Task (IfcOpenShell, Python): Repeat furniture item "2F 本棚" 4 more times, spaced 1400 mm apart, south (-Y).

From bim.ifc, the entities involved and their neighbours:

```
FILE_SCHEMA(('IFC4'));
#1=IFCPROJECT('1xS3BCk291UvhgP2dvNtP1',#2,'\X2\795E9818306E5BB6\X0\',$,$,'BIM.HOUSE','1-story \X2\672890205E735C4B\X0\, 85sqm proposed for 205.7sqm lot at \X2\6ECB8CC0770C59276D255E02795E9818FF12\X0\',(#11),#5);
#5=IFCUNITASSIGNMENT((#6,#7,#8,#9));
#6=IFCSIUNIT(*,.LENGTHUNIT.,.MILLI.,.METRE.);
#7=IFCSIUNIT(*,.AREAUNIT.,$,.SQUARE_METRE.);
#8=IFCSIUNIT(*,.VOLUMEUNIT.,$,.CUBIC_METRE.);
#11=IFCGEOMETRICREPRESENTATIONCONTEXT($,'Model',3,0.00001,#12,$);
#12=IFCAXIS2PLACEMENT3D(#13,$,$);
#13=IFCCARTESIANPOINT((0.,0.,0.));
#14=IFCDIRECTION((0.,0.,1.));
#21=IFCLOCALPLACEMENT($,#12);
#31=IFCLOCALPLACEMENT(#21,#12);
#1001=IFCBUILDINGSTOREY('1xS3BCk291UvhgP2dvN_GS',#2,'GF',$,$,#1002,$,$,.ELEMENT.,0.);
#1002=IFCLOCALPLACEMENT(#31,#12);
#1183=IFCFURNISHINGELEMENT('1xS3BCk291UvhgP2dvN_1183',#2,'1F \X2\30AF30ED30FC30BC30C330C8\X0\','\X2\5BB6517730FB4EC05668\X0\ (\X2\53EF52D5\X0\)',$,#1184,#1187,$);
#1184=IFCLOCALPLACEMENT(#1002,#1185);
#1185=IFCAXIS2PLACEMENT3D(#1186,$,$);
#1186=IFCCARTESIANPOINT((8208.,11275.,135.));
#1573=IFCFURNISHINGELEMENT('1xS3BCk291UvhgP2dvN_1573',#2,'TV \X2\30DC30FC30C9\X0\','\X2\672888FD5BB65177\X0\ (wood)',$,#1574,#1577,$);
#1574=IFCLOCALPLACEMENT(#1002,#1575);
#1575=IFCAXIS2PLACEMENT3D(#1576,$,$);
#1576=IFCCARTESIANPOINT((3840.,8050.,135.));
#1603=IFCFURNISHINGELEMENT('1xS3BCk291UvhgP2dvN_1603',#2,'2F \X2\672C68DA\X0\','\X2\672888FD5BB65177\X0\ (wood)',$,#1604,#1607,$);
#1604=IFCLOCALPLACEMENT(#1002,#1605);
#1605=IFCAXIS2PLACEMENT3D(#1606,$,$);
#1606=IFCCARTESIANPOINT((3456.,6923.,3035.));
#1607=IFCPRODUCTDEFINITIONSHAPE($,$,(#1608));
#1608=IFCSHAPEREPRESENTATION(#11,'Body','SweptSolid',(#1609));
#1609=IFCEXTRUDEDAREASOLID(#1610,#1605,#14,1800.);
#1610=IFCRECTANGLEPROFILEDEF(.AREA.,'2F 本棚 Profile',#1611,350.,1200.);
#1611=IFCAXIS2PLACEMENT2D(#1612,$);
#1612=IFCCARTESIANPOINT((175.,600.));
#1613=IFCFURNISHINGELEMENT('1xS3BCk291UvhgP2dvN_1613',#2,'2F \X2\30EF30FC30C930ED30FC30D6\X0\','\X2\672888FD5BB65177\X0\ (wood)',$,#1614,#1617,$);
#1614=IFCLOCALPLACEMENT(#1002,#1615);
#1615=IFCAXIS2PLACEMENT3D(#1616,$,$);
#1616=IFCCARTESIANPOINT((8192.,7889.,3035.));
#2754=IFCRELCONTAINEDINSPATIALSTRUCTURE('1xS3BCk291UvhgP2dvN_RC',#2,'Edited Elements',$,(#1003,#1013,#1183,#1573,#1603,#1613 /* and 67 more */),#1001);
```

```python
import numpy as np
import ifcopenshell
import ifcopenshell.api.geometry
import ifcopenshell.api.root
import ifcopenshell.util.element
import ifcopenshell.util.placement

model = ifcopenshell.open("bim.ifc")


def reuse_history(source, copy):
    """copy_class also copies each property set's owner history, people and application; keep the originals."""
    for rel in copy.IsDefinedBy:
        if rel.is_a("IfcRelDefinesByProperties") and (history := rel.RelatingPropertyDefinition.OwnerHistory):
            rel.RelatingPropertyDefinition.OwnerHistory = source.OwnerHistory
            ifcopenshell.util.element.remove_deep2(model, history)


source = model.by_guid("1xS3BCk291UvhgP2dvN_1603")
base = ifcopenshell.util.placement.get_local_placement(source.ObjectPlacement)
step = np.array([0.0, -1.0, 0.0]) * 1400.0

for i in range(1, 5):
    copy = ifcopenshell.api.root.copy_class(model, product=source)
    copy.Representation = ifcopenshell.util.element.copy_deep(
        model, source.Representation, exclude=["IfcGeometricRepresentationContext", "IfcRepresentationMap"]
    )
    reuse_history(source, copy)
    matrix = base.copy()
    matrix[:3, 3] += i * step
    print("added at", matrix[:3, 3].round(3) + 0.0)
    ifcopenshell.api.geometry.edit_object_placement(model, product=copy, matrix=matrix, is_si=False)

model.write("bim_updated.ifc")
```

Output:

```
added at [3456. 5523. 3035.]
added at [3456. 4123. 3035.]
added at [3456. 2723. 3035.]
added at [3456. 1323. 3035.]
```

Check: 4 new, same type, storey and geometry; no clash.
